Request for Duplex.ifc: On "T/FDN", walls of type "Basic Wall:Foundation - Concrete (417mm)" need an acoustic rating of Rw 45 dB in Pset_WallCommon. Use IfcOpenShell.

First a look at what the model holds.

```python
import ifcopenshell
import ifcopenshell.util.element

model = ifcopenshell.open("Duplex.ifc")
print(model.schema)
storey = next(s for s in model.by_type("IfcBuildingStorey") if s.Name == "T/FDN")
walls = [e for e in ifcopenshell.util.element.get_decomposition(storey) if e.is_a("IfcWall")]
seen = {}
for e in walls:
    element_type = ifcopenshell.util.element.get_type(e)
    key = (element_type.Name if element_type != e and element_type else None, ifcopenshell.util.element.get_pset(e, "Pset_WallCommon", "AcousticRating"))
    seen[key] = seen.get(key, 0) + 1
for (name, value), count in sorted(seen.items(), key=str):
    print(count, "x", name, "|", value)
```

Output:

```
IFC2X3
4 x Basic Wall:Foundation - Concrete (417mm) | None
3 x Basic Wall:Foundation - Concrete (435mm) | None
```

```python
import ifcopenshell
import ifcopenshell.api.pset
import ifcopenshell.util.element

model = ifcopenshell.open("Duplex.ifc")

storey = next(s for s in model.by_type("IfcBuildingStorey") if s.Name == "T/FDN")
walls = [e for e in ifcopenshell.util.element.get_decomposition(storey) if e.is_a("IfcWall")]

count = 0
for e in walls:
    element_type = ifcopenshell.util.element.get_type(e)
    if element_type in (None, e) or element_type.Name != "Basic Wall:Foundation - Concrete (417mm)":
        continue
    # add_pset returns the element's existing set when there is one.
    pset = ifcopenshell.api.pset.add_pset(model, product=e, name="Pset_WallCommon")
    ifcopenshell.api.pset.edit_pset(model, pset=pset, properties={"AcousticRating": "Rw 45 dB"})
    count += 1

print(count, "walls updated")

model.write("Duplex_edited.ifc")
```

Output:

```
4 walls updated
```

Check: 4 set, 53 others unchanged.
